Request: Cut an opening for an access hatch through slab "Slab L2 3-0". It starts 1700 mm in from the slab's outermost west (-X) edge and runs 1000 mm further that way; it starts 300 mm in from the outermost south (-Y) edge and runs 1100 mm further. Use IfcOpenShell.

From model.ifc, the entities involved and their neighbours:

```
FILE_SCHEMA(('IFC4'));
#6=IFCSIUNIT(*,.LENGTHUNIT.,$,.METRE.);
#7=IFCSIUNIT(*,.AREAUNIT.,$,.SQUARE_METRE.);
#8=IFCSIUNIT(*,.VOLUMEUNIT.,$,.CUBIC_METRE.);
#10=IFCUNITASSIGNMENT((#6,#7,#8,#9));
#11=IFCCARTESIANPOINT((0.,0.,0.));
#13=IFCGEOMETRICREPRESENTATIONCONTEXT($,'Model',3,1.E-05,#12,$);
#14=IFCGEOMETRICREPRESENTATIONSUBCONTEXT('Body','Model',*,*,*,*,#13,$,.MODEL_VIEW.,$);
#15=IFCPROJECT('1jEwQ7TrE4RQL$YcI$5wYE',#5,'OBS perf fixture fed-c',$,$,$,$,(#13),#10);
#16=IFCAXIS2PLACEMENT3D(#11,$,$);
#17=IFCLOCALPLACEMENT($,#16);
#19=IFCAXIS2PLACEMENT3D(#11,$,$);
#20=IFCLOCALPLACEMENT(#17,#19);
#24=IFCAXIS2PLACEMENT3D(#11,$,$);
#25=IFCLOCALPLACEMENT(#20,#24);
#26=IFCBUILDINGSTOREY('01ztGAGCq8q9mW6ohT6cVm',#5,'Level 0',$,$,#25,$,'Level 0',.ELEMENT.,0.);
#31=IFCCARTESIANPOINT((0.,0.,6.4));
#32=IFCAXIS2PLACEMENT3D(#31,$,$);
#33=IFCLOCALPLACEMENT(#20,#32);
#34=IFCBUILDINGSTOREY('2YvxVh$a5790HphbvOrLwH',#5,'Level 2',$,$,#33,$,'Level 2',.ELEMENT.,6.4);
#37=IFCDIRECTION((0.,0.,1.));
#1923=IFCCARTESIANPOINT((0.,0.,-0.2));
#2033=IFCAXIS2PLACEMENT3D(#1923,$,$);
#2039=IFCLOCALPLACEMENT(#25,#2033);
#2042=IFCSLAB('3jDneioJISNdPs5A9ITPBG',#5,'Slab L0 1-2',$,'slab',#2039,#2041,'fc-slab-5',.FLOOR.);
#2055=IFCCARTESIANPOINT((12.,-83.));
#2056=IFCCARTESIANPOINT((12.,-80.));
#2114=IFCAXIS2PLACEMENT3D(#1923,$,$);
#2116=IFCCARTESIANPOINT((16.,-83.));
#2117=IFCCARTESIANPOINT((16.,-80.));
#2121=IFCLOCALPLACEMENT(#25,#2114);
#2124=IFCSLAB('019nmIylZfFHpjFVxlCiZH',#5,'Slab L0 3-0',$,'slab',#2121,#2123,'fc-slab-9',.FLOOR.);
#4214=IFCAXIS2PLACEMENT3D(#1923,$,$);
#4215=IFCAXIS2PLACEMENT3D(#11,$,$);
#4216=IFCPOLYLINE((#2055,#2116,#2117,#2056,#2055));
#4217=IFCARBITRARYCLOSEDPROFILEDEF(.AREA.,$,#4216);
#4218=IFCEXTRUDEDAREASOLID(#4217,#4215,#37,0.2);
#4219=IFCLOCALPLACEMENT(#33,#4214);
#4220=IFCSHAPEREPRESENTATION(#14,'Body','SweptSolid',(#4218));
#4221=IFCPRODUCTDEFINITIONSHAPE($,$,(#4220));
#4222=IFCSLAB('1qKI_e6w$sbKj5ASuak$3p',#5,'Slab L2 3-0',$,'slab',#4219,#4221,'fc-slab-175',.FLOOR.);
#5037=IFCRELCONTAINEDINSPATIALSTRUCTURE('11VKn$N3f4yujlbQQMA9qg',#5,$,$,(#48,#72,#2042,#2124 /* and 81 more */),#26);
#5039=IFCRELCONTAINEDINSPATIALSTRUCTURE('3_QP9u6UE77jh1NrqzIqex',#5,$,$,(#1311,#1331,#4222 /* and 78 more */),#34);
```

```python
import numpy as np
import ifcopenshell
import ifcopenshell.api.feature
import ifcopenshell.api.geometry
import ifcopenshell.api.root
import ifcopenshell.geom
import ifcopenshell.util.placement
import ifcopenshell.util.representation
import ifcopenshell.util.shape
import ifcopenshell.util.unit

model = ifcopenshell.open("model.ifc")
unit_scale = ifcopenshell.util.unit.calculate_unit_scale(model)
settings = ifcopenshell.geom.settings()


def volume(element):
    """Net volume in cubic metres, openings subtracted."""
    shape = ifcopenshell.geom.create_shape(settings, element)
    return ifcopenshell.util.shape.get_volume(shape.geometry)


slab = model.by_guid("1qKI_e6w$sbKj5ASuak$3p")
before = volume(slab)

# Extent in the slab's own axes, in metres. The edges named are its -X and -Y sides.
slab_shape = ifcopenshell.geom.create_shape(settings, slab)
vertices = ifcopenshell.util.shape.get_vertices(slab_shape.geometry)
x_min, y_min, bottom = vertices.min(axis=0)
top = vertices[:, 2].max()

opening = ifcopenshell.api.root.create_entity(model, ifc_class="IfcOpeningElement", name="Access hatch opening", predefined_type="OPENING")
context = ifcopenshell.util.representation.get_context(model, "Model", "Body", "MODEL_VIEW")
width, depth = 1, 1.1
outline = [(0.0, 0.0), (width, 0.0), (width, depth), (0.0, depth), (0.0, 0.0)]
# Overshoot both faces by 50 mm so the cut is clean.
shape = ifcopenshell.api.geometry.add_slab_representation(
    model, context=context, depth=top - bottom + 0.1, polyline=outline
)
ifcopenshell.api.geometry.assign_representation(model, product=opening, representation=shape)

matrix = ifcopenshell.util.placement.get_local_placement(slab.ObjectPlacement)
matrix[:, 3] = matrix @ np.append(np.array([x_min + 1.7, y_min + 0.3, bottom - 0.05]) / unit_scale, 1.0)
ifcopenshell.api.geometry.edit_object_placement(model, product=opening, matrix=matrix, is_si=False)
ifcopenshell.api.feature.add_feature(model, feature=opening, element=slab)

after = volume(slab)

print(f"slab volume {before:.3f} -> {after:.3f} m3")

model.write("model_updated.ifc")
```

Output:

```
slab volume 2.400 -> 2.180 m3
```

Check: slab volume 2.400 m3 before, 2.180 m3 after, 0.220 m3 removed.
